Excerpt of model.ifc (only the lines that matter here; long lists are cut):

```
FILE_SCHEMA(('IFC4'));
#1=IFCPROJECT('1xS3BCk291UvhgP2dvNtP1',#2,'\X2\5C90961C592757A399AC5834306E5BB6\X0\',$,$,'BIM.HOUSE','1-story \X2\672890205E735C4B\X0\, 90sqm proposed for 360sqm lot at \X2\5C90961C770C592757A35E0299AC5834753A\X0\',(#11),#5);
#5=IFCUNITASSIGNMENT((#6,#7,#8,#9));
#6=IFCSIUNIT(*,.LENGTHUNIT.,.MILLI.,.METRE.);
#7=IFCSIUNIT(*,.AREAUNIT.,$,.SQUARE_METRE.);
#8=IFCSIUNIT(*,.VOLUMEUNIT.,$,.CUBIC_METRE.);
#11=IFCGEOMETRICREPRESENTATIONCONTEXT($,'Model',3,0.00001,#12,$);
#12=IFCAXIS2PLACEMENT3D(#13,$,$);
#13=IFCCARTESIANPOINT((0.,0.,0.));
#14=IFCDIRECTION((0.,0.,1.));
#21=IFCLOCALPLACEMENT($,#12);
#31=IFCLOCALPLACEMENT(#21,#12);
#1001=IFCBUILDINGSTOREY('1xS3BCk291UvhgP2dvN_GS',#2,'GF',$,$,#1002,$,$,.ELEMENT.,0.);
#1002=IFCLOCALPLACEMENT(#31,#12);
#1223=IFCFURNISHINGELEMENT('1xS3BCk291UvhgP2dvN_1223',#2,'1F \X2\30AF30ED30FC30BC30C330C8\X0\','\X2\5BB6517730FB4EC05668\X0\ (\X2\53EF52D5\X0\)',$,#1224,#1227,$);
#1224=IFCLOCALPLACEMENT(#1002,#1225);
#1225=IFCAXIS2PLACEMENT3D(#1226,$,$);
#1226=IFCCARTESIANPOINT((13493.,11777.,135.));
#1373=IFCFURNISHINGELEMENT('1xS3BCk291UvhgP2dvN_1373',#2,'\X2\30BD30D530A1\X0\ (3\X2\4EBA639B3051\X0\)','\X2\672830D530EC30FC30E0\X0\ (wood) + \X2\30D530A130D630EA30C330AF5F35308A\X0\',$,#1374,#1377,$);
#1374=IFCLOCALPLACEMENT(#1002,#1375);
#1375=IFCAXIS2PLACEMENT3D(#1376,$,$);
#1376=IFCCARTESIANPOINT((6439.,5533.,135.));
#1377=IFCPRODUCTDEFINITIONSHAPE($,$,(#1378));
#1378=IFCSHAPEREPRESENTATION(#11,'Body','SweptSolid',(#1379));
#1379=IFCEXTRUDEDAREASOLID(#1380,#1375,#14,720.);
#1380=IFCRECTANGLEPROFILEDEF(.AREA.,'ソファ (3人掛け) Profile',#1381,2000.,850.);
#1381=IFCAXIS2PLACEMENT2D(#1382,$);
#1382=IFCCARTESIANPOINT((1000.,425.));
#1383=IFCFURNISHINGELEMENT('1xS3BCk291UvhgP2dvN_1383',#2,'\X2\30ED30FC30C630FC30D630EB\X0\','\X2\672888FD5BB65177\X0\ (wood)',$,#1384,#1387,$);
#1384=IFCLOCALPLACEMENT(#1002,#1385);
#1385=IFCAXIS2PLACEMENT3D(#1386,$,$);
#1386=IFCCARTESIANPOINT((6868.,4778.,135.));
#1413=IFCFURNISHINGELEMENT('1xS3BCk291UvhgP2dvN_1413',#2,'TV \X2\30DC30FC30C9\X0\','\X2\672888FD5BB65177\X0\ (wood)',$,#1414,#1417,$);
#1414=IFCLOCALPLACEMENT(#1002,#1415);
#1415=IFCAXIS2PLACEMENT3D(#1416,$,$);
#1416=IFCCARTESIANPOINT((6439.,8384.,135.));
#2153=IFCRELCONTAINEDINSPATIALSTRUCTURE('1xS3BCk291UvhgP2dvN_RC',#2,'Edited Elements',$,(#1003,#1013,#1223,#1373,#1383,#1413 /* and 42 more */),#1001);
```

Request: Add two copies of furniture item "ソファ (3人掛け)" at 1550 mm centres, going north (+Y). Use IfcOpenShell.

```python
import numpy as np
import ifcopenshell
import ifcopenshell.api.geometry
import ifcopenshell.api.root
import ifcopenshell.util.element
import ifcopenshell.util.placement
import ifcopenshell.util.unit

model = ifcopenshell.open("model.ifc")
unit_scale = ifcopenshell.util.unit.calculate_unit_scale(model)


def reuse_history(source, copy):
    """copy_class also copies each property set's owner history, people and application; keep the originals."""
    for rel in copy.IsDefinedBy:
        if rel.is_a("IfcRelDefinesByProperties") and (history := rel.RelatingPropertyDefinition.OwnerHistory):
            rel.RelatingPropertyDefinition.OwnerHistory = source.OwnerHistory
            ifcopenshell.util.element.remove_deep2(model, history)


source = model.by_id(1373)
base = ifcopenshell.util.placement.get_local_placement(source.ObjectPlacement)
step = np.array([0.0, 1.0, 0.0]) * 1.55 / unit_scale

for i in range(1, 3):
    copy = ifcopenshell.api.root.copy_class(model, product=source)
    copy.Representation = ifcopenshell.util.element.copy_deep(
        model, source.Representation, exclude=["IfcGeometricRepresentationContext", "IfcRepresentationMap"]
    )
    reuse_history(source, copy)
    matrix = base.copy()
    matrix[:3, 3] += i * step
    print("added at", matrix[:3, 3].round(3) + 0.0)
    ifcopenshell.api.geometry.edit_object_placement(model, product=copy, matrix=matrix, is_si=False)

model.write("model_edited.ifc")
```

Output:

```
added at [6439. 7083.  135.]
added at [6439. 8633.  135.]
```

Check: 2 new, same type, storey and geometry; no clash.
